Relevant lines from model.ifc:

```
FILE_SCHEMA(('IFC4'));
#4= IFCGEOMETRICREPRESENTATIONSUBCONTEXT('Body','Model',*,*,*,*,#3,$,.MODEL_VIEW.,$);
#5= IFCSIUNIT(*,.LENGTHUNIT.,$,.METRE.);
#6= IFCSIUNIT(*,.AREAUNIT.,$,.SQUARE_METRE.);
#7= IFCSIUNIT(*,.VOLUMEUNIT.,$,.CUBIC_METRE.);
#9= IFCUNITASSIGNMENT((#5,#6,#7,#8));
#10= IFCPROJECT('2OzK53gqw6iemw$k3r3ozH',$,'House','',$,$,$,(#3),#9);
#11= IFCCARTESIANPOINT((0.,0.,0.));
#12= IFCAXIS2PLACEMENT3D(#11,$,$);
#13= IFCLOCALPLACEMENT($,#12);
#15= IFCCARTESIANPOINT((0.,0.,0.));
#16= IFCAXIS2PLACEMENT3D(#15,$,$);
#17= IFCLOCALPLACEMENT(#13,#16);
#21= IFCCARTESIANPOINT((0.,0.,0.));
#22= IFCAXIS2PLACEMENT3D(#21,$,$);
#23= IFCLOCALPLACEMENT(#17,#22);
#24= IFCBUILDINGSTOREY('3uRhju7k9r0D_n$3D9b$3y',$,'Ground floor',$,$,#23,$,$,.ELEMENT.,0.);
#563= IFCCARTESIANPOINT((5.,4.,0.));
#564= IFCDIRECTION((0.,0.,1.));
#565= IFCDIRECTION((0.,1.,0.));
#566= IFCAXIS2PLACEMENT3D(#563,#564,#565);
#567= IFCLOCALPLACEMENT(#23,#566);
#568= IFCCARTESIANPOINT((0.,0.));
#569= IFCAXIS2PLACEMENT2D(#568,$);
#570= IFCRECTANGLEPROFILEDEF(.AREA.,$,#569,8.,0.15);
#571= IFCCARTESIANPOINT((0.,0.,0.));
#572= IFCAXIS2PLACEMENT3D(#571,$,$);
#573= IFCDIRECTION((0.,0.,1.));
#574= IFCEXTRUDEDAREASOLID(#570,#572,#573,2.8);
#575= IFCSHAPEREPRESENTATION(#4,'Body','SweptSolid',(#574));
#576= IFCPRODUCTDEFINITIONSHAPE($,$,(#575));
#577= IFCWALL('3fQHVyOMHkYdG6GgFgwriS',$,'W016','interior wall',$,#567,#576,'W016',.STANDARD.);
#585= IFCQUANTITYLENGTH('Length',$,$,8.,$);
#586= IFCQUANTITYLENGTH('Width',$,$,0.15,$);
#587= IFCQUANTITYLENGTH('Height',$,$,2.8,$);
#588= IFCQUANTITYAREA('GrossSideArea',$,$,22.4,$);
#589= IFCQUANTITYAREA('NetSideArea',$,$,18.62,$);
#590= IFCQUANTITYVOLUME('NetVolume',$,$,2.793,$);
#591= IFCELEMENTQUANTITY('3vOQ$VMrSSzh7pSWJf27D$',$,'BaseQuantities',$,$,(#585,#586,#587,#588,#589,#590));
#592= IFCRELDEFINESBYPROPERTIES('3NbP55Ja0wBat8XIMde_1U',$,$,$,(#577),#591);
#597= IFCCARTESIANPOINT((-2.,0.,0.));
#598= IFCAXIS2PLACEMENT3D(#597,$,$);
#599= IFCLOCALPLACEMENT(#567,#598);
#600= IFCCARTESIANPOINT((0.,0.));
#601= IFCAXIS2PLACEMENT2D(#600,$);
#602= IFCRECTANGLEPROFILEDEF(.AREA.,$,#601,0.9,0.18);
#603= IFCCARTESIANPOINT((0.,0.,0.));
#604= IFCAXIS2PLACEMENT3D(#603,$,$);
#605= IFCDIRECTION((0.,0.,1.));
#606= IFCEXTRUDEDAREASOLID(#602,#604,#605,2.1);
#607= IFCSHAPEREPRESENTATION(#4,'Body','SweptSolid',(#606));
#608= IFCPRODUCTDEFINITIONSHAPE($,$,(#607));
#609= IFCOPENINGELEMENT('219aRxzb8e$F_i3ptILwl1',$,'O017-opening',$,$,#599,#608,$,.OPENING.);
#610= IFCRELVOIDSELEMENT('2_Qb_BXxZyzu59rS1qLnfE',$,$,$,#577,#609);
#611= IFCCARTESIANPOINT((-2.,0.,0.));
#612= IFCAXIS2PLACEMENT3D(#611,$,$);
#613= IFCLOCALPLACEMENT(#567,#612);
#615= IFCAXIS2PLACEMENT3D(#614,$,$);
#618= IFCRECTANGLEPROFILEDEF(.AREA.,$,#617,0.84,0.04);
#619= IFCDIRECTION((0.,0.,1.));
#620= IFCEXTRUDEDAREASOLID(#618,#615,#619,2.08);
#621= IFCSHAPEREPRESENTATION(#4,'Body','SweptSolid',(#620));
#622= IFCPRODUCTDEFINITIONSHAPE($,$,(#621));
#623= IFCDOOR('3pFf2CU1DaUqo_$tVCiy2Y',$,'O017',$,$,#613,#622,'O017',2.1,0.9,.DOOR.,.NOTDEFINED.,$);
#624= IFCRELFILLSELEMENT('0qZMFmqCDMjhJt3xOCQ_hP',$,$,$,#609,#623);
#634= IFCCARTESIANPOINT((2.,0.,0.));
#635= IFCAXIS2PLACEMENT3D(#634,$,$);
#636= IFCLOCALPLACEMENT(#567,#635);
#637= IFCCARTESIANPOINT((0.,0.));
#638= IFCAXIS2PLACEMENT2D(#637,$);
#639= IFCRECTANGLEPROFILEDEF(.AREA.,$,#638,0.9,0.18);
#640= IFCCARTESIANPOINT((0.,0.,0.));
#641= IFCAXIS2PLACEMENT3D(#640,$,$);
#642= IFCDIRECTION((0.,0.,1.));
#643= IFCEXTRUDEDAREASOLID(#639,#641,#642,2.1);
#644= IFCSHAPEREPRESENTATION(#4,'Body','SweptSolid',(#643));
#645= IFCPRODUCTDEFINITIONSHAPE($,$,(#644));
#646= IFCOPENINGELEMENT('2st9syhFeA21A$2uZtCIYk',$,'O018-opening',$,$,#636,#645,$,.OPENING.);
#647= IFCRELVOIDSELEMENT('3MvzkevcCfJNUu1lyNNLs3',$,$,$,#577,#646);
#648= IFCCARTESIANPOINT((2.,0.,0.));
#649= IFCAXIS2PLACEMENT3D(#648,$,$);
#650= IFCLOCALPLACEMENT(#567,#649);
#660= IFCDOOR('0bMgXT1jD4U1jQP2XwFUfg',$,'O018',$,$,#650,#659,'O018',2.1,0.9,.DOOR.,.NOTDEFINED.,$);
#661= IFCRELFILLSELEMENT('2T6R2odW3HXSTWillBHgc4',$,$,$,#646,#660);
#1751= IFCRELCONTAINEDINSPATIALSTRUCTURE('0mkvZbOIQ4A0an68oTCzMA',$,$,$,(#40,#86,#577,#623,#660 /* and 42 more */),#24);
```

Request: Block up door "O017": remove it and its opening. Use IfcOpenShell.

```python
import ifcopenshell
import ifcopenshell.api.feature
import ifcopenshell.api.pset
import ifcopenshell.api.root
import ifcopenshell.geom
import ifcopenshell.util.element
import ifcopenshell.util.shape
import ifcopenshell.util.unit

model = ifcopenshell.open("model.ifc")
area_scale = ifcopenshell.util.unit.calculate_unit_scale(model, "AREAUNIT")
volume_scale = ifcopenshell.util.unit.calculate_unit_scale(model, "VOLUMEUNIT")
settings = ifcopenshell.geom.settings()


def volume(element):
    """Net volume in cubic metres, openings subtracted."""
    shape = ifcopenshell.geom.create_shape(settings, element)
    return ifcopenshell.util.shape.get_volume(shape.geometry)


door = model.by_id(623)
opening = door.FillsVoids[0].RelatingOpeningElement
wall = opening.VoidsElements[0].RelatingBuildingElement
before = volume(wall)

ifcopenshell.api.root.remove_product(model, product=door)
ifcopenshell.api.feature.remove_feature(model, feature=opening)

after = volume(wall)
thickness = 0.15  # wall thickness in metres

# Update the wall's stored quantities.
qto = model.by_id(ifcopenshell.util.element.get_pset(wall, "BaseQuantities", should_inherit=False)["id"])
ifcopenshell.api.pset.edit_qto(model, qto=qto, properties={
    "NetSideArea": after / thickness / area_scale,
    "NetVolume": after / volume_scale,
})

print(f"wall volume {before:.3f} -> {after:.3f} m3")

model.write("model_v2.ifc")
```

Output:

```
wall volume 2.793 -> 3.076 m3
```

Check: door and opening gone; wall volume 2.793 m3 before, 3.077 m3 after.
